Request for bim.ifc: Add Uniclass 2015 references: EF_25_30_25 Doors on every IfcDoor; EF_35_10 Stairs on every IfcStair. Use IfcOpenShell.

First a look at what the model holds.

```python
import ifcopenshell

model = ifcopenshell.open("bim.ifc")
print(model.schema)
print("classifications:", [c.Name for c in model.by_type("IfcClassification")])
for ifc_class in ("IfcDoor", "IfcRoof", "IfcStair", "IfcWall", "IfcWindow"):
    print(ifc_class, len(model.by_type(ifc_class)))
```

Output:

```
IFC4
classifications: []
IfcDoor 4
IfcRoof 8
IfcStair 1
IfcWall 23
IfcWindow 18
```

```python
import ifcopenshell
import ifcopenshell.api.classification

model = ifcopenshell.open("bim.ifc")

system = ifcopenshell.api.classification.add_classification(model, classification="Uniclass 2015")

codes = {
    "IfcDoor": ("EF_25_30_25", "Doors"),
    "IfcStair": ("EF_35_10", "Stairs"),
}
for ifc_class, (code, name) in codes.items():
    products = model.by_type(ifc_class)
    ifcopenshell.api.classification.add_reference(
        model, products=products, classification=system, identification=code, name=name
    )
    print(code, len(products))

model.write("bim_v2.ifc")
```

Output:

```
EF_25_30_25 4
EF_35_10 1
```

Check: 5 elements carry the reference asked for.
